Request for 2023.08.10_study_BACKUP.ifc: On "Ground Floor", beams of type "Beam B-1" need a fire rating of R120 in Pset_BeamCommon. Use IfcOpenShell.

First a look at what the model holds.

```python
import ifcopenshell
import ifcopenshell.util.element

model = ifcopenshell.open("2023.08.10_study_BACKUP.ifc")
print(model.schema)
storey = next(s for s in model.by_type("IfcBuildingStorey") if s.Name == "Ground Floor")
beams = [e for e in ifcopenshell.util.element.get_decomposition(storey) if e.is_a("IfcBeam")]
seen = {}
for e in beams:
    element_type = ifcopenshell.util.element.get_type(e)
    key = (element_type.Name if element_type != e and element_type else None, ifcopenshell.util.element.get_pset(e, "Pset_BeamCommon", "FireRating"))
    seen[key] = seen.get(key, 0) + 1
for (name, value), count in sorted(seen.items(), key=str):
    print(count, "x", name, "|", value)
```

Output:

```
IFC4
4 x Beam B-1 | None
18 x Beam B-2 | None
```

```python
import ifcopenshell
import ifcopenshell.api.pset
import ifcopenshell.util.element

model = ifcopenshell.open("2023.08.10_study_BACKUP.ifc")

storey = next(s for s in model.by_type("IfcBuildingStorey") if s.Name == "Ground Floor")
beams = [e for e in ifcopenshell.util.element.get_decomposition(storey) if e.is_a("IfcBeam")]

count = 0
for e in beams:
    element_type = ifcopenshell.util.element.get_type(e)
    if element_type in (None, e) or element_type.Name != "Beam B-1":
        continue
    # add_pset returns the element's existing set when there is one.
    pset = ifcopenshell.api.pset.add_pset(model, product=e, name="Pset_BeamCommon")
    ifcopenshell.api.pset.edit_pset(model, pset=pset, properties={"FireRating": "R120"})
    count += 1

print(count, "beams updated")

model.write("2023.08.10_study_BACKUP_v2.ifc")
```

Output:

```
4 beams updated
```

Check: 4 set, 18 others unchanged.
